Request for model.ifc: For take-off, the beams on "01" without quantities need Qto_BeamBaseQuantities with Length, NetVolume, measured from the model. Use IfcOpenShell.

First a look at what the model holds.

```python
import ifcopenshell
import ifcopenshell.util.element
import ifcopenshell.util.unit

model = ifcopenshell.open("model.ifc")
print(model.schema)
for unit_type in ("LENGTHUNIT", "AREAUNIT", "VOLUMEUNIT"):
    print(unit_type, ifcopenshell.util.unit.calculate_unit_scale(model, unit_type))
storey = next(s for s in model.by_type("IfcBuildingStorey") if s.Name == "01")
beams = [e for e in ifcopenshell.util.element.get_decomposition(storey) if e.is_a("IfcBeam")]
for e in sorted(beams, key=lambda e: e.id()):
    print(e.id(), e.is_a(), e.Name, list(ifcopenshell.util.element.get_psets(e, qtos_only=True)), sep=" | ")
```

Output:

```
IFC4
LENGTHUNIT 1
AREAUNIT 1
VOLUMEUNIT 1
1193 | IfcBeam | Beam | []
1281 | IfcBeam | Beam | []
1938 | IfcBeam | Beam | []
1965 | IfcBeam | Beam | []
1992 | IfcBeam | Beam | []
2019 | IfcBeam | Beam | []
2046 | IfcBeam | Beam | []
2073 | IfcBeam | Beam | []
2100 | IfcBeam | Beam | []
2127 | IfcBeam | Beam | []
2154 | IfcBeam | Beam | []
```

```python
import ifcopenshell
import ifcopenshell.api.pset
import ifcopenshell.geom
import ifcopenshell.util.element
import ifcopenshell.util.shape
import ifcopenshell.util.unit

model = ifcopenshell.open("model.ifc")
unit_scale = ifcopenshell.util.unit.calculate_unit_scale(model)
volume_scale = ifcopenshell.util.unit.calculate_unit_scale(model, "VOLUMEUNIT")
settings = ifcopenshell.geom.settings()

storey = next(s for s in model.by_type("IfcBuildingStorey") if s.Name == "01")
beams = [e for e in ifcopenshell.util.element.get_decomposition(storey) if e.is_a("IfcBeam")]

for e in sorted(beams, key=lambda e: e.id()):
    if ifcopenshell.util.element.get_psets(e, qtos_only=True, should_inherit=False):
        continue
    # Geometry comes back in metres, in the element's own axes.
    shape = ifcopenshell.geom.create_shape(settings, e)
    values = {
        "Length": ifcopenshell.util.shape.get_max_xyz(shape.geometry) / unit_scale,
        "NetVolume": ifcopenshell.util.shape.get_volume(shape.geometry) / volume_scale,
    }
    qto = ifcopenshell.api.pset.add_qto(model, product=e, name="Qto_BeamBaseQuantities")
    ifcopenshell.api.pset.edit_qto(model, qto=qto, properties=values)
    print(e.id(), {k: round(v, 3) for k, v in values.items()})

model.write("model_v2.ifc")
```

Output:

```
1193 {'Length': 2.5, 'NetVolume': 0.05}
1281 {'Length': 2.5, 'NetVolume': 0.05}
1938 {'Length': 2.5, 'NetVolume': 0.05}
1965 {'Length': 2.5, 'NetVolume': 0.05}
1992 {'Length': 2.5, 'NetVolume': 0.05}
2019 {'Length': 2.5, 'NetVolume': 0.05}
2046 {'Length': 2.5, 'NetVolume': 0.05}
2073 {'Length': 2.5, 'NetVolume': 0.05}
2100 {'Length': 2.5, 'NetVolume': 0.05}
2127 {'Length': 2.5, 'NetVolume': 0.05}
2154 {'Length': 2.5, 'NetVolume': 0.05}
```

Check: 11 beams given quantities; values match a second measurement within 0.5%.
